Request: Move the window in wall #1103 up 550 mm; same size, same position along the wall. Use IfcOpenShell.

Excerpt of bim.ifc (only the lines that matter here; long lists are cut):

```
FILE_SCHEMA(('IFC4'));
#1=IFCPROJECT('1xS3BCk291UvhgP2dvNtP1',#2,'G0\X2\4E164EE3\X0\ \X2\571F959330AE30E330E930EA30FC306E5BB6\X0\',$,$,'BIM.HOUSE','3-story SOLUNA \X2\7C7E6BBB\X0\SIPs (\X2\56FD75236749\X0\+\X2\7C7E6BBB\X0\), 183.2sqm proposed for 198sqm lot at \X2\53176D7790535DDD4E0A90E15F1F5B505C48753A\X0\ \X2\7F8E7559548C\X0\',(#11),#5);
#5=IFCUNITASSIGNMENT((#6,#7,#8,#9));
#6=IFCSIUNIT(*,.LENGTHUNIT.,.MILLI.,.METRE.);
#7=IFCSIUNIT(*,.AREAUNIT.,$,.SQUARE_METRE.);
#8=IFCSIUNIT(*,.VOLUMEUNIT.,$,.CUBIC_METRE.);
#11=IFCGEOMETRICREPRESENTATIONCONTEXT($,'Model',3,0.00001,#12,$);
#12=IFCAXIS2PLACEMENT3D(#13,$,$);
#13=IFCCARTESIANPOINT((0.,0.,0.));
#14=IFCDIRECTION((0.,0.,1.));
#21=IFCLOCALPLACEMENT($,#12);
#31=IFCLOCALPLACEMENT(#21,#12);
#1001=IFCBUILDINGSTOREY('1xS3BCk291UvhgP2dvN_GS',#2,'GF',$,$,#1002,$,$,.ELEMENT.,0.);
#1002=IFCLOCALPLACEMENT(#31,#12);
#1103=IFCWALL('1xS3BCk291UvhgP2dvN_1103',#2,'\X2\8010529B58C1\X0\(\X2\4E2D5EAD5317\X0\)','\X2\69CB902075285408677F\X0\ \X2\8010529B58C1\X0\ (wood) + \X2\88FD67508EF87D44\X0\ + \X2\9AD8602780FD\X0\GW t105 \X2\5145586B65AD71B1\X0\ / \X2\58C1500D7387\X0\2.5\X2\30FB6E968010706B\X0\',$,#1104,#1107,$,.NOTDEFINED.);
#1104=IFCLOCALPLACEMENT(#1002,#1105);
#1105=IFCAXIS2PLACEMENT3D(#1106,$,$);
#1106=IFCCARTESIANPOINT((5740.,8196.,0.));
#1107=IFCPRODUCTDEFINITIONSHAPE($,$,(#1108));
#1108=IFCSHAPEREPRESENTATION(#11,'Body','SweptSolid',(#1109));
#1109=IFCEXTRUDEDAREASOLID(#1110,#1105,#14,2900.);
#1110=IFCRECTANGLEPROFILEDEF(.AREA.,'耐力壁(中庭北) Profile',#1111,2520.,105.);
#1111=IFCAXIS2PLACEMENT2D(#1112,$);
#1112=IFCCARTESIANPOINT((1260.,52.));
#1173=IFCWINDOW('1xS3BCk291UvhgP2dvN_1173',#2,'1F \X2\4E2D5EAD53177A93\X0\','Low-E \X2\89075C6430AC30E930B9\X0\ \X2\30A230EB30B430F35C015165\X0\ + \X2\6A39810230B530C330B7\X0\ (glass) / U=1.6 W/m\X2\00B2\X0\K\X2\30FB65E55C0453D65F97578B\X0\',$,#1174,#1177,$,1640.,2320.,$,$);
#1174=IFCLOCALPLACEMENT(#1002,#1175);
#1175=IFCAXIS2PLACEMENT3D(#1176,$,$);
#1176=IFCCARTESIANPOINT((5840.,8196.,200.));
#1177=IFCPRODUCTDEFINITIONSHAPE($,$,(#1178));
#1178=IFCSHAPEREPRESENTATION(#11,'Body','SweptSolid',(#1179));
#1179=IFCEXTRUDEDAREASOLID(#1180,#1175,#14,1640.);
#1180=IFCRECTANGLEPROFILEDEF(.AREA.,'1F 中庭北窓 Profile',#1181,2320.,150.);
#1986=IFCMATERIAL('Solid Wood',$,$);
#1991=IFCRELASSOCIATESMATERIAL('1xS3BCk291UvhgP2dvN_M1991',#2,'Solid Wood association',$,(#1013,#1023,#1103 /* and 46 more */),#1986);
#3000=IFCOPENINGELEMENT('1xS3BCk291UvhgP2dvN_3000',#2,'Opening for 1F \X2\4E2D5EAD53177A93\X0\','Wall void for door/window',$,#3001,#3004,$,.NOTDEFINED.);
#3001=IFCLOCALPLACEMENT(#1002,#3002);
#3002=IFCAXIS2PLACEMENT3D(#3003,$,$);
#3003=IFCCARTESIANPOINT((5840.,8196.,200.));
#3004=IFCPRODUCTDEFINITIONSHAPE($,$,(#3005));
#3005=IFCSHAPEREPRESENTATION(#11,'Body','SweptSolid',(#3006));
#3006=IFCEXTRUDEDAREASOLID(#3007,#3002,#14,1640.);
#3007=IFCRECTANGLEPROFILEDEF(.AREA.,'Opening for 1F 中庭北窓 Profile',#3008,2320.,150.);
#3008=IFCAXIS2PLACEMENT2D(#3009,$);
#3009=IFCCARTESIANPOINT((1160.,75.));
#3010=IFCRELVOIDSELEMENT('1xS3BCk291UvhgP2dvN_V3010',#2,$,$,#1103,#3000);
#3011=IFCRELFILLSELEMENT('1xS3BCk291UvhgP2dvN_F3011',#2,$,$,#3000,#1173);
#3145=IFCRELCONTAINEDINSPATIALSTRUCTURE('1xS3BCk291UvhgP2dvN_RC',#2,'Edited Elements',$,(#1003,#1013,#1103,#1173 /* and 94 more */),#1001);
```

```python
import numpy as np
import ifcopenshell
import ifcopenshell.api.geometry
import ifcopenshell.util.placement
import ifcopenshell.util.unit

model = ifcopenshell.open("bim.ifc")
unit_scale = ifcopenshell.util.unit.calculate_unit_scale(model)

window = model.by_guid("1xS3BCk291UvhgP2dvN_1173")
opening = window.FillsVoids[0].RelatingOpeningElement
dz = 0.55 / unit_scale

shift = np.array([0.0, 0.0, dz])
# The window is not placed relative to its opening, so move both.
for product in (opening, window):
    matrix = ifcopenshell.util.placement.get_local_placement(product.ObjectPlacement)
    matrix[:3, 3] += shift
    ifcopenshell.api.geometry.edit_object_placement(model, product=product, matrix=matrix, is_si=False)

print(f"moved by {dz * unit_scale:+.3f} m")

model.write("bim_v2.ifc")
```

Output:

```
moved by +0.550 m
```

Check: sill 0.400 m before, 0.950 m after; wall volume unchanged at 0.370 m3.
